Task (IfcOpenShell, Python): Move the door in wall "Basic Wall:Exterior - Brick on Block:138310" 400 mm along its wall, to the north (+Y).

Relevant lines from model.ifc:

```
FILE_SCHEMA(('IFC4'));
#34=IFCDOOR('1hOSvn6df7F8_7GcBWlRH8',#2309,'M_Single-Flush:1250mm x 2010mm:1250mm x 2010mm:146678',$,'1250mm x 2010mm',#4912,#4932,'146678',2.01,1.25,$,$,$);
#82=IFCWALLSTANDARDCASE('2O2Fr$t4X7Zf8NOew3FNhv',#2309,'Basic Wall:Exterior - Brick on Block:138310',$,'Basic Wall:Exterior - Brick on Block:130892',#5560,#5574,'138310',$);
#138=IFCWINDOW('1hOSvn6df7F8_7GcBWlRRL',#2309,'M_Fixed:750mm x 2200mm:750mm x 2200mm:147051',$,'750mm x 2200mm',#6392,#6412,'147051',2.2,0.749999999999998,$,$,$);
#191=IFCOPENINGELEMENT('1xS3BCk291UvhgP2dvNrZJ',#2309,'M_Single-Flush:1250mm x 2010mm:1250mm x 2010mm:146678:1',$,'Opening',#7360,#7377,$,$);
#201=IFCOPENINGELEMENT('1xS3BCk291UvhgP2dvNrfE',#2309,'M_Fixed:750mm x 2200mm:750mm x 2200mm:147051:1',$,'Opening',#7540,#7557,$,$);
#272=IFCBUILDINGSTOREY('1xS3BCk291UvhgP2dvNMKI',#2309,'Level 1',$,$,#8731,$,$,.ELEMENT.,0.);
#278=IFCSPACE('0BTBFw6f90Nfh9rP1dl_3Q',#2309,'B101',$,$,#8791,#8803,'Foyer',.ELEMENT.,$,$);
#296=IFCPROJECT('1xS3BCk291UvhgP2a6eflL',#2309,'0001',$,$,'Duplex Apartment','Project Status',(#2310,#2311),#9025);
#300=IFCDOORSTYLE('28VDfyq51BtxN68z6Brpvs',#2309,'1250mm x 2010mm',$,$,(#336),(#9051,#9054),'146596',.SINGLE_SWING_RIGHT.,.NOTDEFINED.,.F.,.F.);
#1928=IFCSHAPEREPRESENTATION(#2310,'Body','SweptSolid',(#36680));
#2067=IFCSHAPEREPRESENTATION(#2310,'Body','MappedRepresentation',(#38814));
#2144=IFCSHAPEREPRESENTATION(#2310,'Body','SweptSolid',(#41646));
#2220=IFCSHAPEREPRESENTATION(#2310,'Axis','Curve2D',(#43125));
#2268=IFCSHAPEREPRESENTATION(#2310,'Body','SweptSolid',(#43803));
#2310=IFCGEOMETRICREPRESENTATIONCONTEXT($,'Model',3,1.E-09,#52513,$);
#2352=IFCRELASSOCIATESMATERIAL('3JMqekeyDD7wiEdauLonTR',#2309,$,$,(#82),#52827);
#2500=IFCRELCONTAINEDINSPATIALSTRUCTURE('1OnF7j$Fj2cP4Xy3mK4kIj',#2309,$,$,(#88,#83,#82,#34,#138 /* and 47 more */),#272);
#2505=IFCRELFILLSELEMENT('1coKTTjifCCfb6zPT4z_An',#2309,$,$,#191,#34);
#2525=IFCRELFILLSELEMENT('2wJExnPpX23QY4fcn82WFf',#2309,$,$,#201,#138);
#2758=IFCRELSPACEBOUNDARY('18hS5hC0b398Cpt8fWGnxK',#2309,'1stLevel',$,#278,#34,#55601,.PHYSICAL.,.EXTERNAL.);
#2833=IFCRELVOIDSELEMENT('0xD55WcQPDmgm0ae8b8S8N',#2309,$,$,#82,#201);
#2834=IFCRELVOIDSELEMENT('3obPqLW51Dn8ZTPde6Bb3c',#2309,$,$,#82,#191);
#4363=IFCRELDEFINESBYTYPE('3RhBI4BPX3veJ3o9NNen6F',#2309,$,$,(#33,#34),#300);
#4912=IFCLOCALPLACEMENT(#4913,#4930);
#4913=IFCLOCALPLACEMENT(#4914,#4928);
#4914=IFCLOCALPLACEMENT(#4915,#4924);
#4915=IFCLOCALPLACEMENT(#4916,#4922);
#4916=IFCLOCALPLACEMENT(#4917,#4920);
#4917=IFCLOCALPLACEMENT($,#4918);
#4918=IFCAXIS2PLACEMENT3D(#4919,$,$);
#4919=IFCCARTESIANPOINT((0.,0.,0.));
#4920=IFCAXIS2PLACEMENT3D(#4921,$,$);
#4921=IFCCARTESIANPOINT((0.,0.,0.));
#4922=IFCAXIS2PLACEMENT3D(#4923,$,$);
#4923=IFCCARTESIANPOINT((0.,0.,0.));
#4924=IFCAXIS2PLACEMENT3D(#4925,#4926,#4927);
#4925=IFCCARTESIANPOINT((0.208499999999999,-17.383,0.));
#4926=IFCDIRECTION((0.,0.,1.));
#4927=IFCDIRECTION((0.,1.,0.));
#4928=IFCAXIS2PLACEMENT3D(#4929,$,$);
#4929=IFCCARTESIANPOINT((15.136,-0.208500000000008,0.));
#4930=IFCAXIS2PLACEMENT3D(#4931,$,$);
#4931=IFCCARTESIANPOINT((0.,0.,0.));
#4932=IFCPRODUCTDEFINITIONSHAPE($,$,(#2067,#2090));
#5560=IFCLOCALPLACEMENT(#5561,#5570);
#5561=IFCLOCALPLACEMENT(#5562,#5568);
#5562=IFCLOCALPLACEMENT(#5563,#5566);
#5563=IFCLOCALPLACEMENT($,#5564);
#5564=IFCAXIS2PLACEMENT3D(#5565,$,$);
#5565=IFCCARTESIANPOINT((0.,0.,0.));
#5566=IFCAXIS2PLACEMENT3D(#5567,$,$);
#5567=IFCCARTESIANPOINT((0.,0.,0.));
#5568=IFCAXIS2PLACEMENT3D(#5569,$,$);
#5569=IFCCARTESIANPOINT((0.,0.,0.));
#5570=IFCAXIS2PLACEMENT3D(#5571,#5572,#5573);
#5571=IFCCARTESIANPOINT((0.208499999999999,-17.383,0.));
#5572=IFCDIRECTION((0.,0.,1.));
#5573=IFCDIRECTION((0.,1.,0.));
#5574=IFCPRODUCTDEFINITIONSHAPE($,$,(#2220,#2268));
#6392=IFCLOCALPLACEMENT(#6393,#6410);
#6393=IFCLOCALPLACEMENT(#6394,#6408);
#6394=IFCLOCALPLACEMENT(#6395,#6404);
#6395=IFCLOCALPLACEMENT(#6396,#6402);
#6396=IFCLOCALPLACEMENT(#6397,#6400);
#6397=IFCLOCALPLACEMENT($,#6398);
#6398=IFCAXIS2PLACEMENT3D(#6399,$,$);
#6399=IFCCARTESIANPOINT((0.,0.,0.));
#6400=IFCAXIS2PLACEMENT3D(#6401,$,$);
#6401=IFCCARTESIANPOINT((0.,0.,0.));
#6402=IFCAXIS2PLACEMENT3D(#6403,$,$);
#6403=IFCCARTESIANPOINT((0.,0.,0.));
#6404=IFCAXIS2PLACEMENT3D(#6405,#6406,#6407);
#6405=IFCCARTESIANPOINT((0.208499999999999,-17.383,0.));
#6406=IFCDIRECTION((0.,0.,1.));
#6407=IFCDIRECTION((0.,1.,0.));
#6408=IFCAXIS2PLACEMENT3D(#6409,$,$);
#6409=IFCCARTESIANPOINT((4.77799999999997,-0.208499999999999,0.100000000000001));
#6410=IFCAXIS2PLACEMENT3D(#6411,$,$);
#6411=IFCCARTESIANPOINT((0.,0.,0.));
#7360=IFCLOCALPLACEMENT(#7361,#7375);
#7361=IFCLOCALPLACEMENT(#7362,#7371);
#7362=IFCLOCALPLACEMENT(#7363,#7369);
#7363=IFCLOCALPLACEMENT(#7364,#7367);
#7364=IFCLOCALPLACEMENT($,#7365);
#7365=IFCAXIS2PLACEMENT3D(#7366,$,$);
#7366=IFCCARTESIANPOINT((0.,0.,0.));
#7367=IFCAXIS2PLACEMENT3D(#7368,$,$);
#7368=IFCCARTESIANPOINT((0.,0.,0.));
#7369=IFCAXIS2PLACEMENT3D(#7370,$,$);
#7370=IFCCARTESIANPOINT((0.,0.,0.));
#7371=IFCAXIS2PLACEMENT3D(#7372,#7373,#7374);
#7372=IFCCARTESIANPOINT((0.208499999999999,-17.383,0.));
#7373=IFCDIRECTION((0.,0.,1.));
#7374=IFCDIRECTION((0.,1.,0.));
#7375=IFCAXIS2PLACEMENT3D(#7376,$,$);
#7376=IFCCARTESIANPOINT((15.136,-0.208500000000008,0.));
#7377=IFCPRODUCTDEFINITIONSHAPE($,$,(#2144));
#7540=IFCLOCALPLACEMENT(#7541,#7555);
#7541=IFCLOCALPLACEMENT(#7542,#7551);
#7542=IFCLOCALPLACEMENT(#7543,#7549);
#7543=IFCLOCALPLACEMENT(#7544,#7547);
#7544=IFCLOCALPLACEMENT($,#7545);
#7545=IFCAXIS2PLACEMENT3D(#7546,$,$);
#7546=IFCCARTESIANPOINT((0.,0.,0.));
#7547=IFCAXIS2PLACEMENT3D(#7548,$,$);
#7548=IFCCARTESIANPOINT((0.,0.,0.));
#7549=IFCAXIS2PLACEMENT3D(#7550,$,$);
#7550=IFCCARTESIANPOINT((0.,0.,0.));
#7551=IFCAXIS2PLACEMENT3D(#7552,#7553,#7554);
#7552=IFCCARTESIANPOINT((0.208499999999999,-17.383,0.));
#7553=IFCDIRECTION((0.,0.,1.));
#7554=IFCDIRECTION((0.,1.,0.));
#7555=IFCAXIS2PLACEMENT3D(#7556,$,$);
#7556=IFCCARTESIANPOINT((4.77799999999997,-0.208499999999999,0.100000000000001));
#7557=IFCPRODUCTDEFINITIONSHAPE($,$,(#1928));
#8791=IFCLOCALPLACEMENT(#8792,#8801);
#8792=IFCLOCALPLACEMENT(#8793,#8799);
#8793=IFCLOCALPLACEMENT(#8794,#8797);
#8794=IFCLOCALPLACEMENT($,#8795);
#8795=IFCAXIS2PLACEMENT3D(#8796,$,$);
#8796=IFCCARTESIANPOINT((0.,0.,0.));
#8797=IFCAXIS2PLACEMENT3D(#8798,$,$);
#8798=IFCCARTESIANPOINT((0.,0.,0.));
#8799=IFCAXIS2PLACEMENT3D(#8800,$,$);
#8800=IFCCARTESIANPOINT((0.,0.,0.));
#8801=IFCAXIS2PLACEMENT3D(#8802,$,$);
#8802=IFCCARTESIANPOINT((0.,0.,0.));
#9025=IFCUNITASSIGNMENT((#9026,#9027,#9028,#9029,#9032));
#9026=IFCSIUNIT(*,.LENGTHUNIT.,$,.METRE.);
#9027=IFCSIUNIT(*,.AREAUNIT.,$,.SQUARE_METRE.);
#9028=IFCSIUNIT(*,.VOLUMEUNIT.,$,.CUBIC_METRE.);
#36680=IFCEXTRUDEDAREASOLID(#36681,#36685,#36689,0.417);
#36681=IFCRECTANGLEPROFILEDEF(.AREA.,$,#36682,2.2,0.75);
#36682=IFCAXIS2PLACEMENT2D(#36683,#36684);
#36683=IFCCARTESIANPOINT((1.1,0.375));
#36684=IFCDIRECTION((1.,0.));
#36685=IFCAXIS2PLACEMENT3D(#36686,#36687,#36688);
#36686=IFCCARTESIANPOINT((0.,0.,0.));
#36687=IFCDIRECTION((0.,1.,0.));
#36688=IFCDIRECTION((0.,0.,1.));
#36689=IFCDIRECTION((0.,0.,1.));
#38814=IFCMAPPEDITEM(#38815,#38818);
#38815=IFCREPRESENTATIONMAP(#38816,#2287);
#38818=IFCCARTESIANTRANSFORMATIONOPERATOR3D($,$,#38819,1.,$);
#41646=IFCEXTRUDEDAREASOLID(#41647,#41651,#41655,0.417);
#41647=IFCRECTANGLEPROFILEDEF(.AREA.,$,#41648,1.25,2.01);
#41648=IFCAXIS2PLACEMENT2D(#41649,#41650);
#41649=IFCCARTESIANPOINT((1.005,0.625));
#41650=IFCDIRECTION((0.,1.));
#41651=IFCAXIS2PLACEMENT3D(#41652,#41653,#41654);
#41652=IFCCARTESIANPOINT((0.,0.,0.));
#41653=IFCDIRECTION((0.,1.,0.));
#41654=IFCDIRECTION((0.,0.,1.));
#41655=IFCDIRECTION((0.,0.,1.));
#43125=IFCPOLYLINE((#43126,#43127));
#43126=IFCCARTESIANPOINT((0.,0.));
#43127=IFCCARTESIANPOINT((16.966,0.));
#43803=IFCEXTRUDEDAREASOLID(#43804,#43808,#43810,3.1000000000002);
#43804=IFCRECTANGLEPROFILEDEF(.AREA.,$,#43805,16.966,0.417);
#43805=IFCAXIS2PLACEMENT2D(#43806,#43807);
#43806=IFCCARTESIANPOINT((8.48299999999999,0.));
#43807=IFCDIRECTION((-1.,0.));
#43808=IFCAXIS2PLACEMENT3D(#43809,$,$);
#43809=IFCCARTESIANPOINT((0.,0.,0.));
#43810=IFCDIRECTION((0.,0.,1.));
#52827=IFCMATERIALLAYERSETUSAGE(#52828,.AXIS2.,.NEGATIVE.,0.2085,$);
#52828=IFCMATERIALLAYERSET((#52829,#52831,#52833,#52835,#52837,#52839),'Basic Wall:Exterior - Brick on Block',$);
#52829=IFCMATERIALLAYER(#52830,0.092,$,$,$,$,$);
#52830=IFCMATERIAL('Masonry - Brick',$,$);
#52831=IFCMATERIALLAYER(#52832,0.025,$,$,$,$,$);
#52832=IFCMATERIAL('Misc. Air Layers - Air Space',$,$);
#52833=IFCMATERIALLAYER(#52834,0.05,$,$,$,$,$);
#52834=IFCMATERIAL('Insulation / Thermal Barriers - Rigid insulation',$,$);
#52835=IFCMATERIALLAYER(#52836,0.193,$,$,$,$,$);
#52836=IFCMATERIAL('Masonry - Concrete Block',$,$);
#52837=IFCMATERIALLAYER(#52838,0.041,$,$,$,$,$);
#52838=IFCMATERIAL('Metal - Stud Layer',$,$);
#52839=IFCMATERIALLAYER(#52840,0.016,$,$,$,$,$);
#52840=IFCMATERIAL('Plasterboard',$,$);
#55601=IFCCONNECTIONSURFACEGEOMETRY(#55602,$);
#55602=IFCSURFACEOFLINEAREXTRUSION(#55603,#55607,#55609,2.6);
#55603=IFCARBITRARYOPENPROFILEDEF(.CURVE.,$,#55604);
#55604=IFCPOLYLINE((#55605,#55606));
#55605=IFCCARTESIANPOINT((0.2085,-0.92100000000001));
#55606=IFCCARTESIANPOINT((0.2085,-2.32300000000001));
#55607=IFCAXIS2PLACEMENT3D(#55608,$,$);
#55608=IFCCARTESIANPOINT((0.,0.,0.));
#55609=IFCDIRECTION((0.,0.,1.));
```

```python
import numpy as np
import ifcopenshell
import ifcopenshell.api.geometry
import ifcopenshell.util.placement

model = ifcopenshell.open("model.ifc")

door = model.by_guid("1hOSvn6df7F8_7GcBWlRH8")
opening = door.FillsVoids[0].RelatingOpeningElement
wall = opening.VoidsElements[0].RelatingBuildingElement

wall_matrix = ifcopenshell.util.placement.get_local_placement(wall.ObjectPlacement)
shift = wall_matrix[:3, 0] * 0.4
before = ifcopenshell.util.placement.get_local_placement(door.ObjectPlacement)[:3, 3].copy()

# The door is not placed relative to its opening, so move both.
for product in (opening, door):
    matrix = ifcopenshell.util.placement.get_local_placement(product.ObjectPlacement)
    matrix[:3, 3] += shift
    ifcopenshell.api.geometry.edit_object_placement(model, product=product, matrix=matrix, is_si=False)

# Space boundary surfaces are stored in each space's coordinates; move them too.
for rel in door.ProvidesBoundaries:
    if not rel.ConnectionGeometry:
        continue
    surface = rel.ConnectionGeometry.SurfaceOnRelatingElement
    space_matrix = ifcopenshell.util.placement.get_local_placement(rel.RelatingSpace.ObjectPlacement)
    point = np.array(surface.Position.Location.Coordinates) + space_matrix[:3, :3].T @ shift
    surface.Position = model.createIfcAxis2Placement3D(
        model.createIfcCartesianPoint(point.tolist()), surface.Position.Axis, surface.Position.RefDirection
    )

after = ifcopenshell.util.placement.get_local_placement(door.ObjectPlacement)[:3, 3]
print("door moved by", (after - before).round(3) + 0.0)

model.write("model_updated.ifc")
```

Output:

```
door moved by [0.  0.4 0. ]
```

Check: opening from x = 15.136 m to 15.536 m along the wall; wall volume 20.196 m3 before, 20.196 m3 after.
